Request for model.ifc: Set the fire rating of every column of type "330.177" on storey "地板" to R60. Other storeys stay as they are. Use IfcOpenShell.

First a look at what the model holds.

```python
import ifcopenshell
import ifcopenshell.util.element

model = ifcopenshell.open("model.ifc")
print(model.schema)
storey = next(s for s in model.by_type("IfcBuildingStorey") if s.Name == "地板")
columns = [e for e in ifcopenshell.util.element.get_decomposition(storey) if e.is_a("IfcColumn")]
seen = {}
for e in columns:
    element_type = ifcopenshell.util.element.get_type(e)
    key = (element_type.Name if element_type != e and element_type else None, ifcopenshell.util.element.get_pset(e, "Pset_ColumnCommon", "FireRating"))
    seen[key] = seen.get(key, 0) + 1
for (name, value), count in sorted(seen.items(), key=str):
    print(count, "x", name, "|", value)
```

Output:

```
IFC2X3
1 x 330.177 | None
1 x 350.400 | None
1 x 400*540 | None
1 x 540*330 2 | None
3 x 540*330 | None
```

```python
import ifcopenshell
import ifcopenshell.api.pset
import ifcopenshell.util.element

model = ifcopenshell.open("model.ifc")

storey = next(s for s in model.by_type("IfcBuildingStorey") if s.Name == "地板")
columns = [e for e in ifcopenshell.util.element.get_decomposition(storey) if e.is_a("IfcColumn")]

count = 0
for e in columns:
    element_type = ifcopenshell.util.element.get_type(e)
    if element_type in (None, e) or element_type.Name != "330.177":
        continue
    # add_pset returns the element's existing set when there is one.
    pset = ifcopenshell.api.pset.add_pset(model, product=e, name="Pset_ColumnCommon")
    ifcopenshell.api.pset.edit_pset(model, pset=pset, properties={"FireRating": "R60"})
    count += 1

print(count, "columns updated")

model.write("model_edited.ifc")
```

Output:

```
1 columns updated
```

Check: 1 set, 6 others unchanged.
